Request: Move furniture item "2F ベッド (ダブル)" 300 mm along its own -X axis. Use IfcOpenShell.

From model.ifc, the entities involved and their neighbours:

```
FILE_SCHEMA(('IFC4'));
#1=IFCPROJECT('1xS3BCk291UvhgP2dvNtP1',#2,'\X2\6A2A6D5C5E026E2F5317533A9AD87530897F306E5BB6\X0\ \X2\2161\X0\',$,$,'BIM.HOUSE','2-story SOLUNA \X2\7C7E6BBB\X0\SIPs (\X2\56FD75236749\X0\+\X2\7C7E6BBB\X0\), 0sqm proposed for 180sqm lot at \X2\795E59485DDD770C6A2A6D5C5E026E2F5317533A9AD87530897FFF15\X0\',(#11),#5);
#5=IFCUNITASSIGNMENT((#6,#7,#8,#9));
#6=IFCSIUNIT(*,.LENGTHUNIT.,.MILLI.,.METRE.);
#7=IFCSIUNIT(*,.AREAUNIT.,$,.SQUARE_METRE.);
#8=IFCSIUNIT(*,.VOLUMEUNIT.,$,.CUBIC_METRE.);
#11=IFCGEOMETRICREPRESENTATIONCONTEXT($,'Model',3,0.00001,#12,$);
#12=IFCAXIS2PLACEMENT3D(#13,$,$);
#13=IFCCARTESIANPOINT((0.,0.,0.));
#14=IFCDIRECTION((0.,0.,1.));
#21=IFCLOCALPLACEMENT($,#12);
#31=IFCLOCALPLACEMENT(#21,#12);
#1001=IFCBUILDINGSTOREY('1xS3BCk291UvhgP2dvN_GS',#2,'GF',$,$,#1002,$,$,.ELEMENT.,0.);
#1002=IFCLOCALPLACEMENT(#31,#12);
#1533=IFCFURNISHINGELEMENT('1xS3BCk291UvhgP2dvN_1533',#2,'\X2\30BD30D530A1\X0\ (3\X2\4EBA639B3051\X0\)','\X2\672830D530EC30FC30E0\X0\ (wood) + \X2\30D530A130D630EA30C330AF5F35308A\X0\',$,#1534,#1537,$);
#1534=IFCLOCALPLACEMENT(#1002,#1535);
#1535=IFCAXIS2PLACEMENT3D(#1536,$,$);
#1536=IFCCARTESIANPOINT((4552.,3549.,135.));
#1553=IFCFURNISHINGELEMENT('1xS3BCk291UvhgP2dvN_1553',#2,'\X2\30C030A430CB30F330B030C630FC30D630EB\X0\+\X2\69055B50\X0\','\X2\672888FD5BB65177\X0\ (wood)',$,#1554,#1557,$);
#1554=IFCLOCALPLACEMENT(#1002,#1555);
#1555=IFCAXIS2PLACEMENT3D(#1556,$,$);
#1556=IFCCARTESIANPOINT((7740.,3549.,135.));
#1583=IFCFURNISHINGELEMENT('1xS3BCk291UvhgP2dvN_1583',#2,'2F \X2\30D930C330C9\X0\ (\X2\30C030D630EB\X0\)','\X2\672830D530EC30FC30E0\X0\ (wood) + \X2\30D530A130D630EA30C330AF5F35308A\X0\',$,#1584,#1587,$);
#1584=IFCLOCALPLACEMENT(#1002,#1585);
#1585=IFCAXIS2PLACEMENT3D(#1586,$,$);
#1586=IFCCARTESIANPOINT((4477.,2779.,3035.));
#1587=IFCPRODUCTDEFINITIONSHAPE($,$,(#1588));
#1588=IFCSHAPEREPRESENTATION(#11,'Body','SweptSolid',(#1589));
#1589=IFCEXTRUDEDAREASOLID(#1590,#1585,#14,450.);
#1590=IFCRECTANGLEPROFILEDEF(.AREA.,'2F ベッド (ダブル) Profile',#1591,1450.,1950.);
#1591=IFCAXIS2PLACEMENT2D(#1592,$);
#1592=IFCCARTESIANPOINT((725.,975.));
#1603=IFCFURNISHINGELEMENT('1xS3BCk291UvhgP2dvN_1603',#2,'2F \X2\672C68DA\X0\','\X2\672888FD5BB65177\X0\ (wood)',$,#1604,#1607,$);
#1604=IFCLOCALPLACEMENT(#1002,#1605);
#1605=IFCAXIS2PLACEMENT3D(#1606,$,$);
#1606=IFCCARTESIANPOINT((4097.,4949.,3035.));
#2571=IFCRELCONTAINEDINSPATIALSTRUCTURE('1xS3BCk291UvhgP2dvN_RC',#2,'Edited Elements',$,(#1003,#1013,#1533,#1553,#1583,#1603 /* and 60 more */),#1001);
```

```python
import ifcopenshell
import ifcopenshell.api.geometry
import ifcopenshell.util.placement
import ifcopenshell.util.unit

model = ifcopenshell.open("model.ifc")
unit_scale = ifcopenshell.util.unit.calculate_unit_scale(model)

item = model.by_guid("1xS3BCk291UvhgP2dvN_1583")
matrix = ifcopenshell.util.placement.get_local_placement(item.ObjectPlacement)
matrix[:3, 3] -= matrix[:3, 0] * 0.3 / unit_scale
ifcopenshell.api.geometry.edit_object_placement(model, product=item, matrix=matrix, is_si=False)

print(ifcopenshell.util.placement.get_local_placement(item.ObjectPlacement).round(3) + 0.0)

model.write("model_rev.ifc")
```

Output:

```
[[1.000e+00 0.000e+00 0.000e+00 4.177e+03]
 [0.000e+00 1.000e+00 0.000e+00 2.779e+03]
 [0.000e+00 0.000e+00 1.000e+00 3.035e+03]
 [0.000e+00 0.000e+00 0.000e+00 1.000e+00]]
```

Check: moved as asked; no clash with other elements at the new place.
